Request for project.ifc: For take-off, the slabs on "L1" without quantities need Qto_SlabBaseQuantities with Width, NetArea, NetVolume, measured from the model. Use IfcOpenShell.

First a look at what the model holds.

```python
import ifcopenshell
import ifcopenshell.util.element
import ifcopenshell.util.unit

model = ifcopenshell.open("project.ifc")
print(model.schema)
for unit_type in ("LENGTHUNIT", "AREAUNIT", "VOLUMEUNIT"):
    print(unit_type, ifcopenshell.util.unit.calculate_unit_scale(model, unit_type))
storey = next(s for s in model.by_type("IfcBuildingStorey") if s.Name == "L1")
slabs = [e for e in ifcopenshell.util.element.get_decomposition(storey) if e.is_a("IfcSlab")]
for e in sorted(slabs, key=lambda e: e.id()):
    print(e.id(), e.is_a(), e.Name, list(ifcopenshell.util.element.get_psets(e, qtos_only=True)), sep=" | ")
```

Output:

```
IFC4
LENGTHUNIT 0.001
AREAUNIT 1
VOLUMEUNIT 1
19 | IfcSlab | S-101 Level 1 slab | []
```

```python
import ifcopenshell
import ifcopenshell.api.pset
import ifcopenshell.geom
import ifcopenshell.util.element
import ifcopenshell.util.shape
import ifcopenshell.util.unit

model = ifcopenshell.open("project.ifc")
unit_scale = ifcopenshell.util.unit.calculate_unit_scale(model)
area_scale = ifcopenshell.util.unit.calculate_unit_scale(model, "AREAUNIT")
volume_scale = ifcopenshell.util.unit.calculate_unit_scale(model, "VOLUMEUNIT")
settings = ifcopenshell.geom.settings()

storey = next(s for s in model.by_type("IfcBuildingStorey") if s.Name == "L1")
slabs = [e for e in ifcopenshell.util.element.get_decomposition(storey) if e.is_a("IfcSlab")]

for e in sorted(slabs, key=lambda e: e.id()):
    if ifcopenshell.util.element.get_psets(e, qtos_only=True, should_inherit=False):
        continue
    # Geometry comes back in metres, in the element's own axes.
    shape = ifcopenshell.geom.create_shape(settings, e)
    values = {
        "Width": ifcopenshell.util.shape.get_z(shape.geometry) / unit_scale,
        "NetArea": ifcopenshell.util.shape.get_footprint_area(shape.geometry) / area_scale,
        "NetVolume": ifcopenshell.util.shape.get_volume(shape.geometry) / volume_scale,
    }
    qto = ifcopenshell.api.pset.add_qto(model, product=e, name="Qto_SlabBaseQuantities")
    ifcopenshell.api.pset.edit_qto(model, qto=qto, properties=values)
    print(e.id(), {k: round(v, 3) for k, v in values.items()})

model.write("project-out.ifc")
```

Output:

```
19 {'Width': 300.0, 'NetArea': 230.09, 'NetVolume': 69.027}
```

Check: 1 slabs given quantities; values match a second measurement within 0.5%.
